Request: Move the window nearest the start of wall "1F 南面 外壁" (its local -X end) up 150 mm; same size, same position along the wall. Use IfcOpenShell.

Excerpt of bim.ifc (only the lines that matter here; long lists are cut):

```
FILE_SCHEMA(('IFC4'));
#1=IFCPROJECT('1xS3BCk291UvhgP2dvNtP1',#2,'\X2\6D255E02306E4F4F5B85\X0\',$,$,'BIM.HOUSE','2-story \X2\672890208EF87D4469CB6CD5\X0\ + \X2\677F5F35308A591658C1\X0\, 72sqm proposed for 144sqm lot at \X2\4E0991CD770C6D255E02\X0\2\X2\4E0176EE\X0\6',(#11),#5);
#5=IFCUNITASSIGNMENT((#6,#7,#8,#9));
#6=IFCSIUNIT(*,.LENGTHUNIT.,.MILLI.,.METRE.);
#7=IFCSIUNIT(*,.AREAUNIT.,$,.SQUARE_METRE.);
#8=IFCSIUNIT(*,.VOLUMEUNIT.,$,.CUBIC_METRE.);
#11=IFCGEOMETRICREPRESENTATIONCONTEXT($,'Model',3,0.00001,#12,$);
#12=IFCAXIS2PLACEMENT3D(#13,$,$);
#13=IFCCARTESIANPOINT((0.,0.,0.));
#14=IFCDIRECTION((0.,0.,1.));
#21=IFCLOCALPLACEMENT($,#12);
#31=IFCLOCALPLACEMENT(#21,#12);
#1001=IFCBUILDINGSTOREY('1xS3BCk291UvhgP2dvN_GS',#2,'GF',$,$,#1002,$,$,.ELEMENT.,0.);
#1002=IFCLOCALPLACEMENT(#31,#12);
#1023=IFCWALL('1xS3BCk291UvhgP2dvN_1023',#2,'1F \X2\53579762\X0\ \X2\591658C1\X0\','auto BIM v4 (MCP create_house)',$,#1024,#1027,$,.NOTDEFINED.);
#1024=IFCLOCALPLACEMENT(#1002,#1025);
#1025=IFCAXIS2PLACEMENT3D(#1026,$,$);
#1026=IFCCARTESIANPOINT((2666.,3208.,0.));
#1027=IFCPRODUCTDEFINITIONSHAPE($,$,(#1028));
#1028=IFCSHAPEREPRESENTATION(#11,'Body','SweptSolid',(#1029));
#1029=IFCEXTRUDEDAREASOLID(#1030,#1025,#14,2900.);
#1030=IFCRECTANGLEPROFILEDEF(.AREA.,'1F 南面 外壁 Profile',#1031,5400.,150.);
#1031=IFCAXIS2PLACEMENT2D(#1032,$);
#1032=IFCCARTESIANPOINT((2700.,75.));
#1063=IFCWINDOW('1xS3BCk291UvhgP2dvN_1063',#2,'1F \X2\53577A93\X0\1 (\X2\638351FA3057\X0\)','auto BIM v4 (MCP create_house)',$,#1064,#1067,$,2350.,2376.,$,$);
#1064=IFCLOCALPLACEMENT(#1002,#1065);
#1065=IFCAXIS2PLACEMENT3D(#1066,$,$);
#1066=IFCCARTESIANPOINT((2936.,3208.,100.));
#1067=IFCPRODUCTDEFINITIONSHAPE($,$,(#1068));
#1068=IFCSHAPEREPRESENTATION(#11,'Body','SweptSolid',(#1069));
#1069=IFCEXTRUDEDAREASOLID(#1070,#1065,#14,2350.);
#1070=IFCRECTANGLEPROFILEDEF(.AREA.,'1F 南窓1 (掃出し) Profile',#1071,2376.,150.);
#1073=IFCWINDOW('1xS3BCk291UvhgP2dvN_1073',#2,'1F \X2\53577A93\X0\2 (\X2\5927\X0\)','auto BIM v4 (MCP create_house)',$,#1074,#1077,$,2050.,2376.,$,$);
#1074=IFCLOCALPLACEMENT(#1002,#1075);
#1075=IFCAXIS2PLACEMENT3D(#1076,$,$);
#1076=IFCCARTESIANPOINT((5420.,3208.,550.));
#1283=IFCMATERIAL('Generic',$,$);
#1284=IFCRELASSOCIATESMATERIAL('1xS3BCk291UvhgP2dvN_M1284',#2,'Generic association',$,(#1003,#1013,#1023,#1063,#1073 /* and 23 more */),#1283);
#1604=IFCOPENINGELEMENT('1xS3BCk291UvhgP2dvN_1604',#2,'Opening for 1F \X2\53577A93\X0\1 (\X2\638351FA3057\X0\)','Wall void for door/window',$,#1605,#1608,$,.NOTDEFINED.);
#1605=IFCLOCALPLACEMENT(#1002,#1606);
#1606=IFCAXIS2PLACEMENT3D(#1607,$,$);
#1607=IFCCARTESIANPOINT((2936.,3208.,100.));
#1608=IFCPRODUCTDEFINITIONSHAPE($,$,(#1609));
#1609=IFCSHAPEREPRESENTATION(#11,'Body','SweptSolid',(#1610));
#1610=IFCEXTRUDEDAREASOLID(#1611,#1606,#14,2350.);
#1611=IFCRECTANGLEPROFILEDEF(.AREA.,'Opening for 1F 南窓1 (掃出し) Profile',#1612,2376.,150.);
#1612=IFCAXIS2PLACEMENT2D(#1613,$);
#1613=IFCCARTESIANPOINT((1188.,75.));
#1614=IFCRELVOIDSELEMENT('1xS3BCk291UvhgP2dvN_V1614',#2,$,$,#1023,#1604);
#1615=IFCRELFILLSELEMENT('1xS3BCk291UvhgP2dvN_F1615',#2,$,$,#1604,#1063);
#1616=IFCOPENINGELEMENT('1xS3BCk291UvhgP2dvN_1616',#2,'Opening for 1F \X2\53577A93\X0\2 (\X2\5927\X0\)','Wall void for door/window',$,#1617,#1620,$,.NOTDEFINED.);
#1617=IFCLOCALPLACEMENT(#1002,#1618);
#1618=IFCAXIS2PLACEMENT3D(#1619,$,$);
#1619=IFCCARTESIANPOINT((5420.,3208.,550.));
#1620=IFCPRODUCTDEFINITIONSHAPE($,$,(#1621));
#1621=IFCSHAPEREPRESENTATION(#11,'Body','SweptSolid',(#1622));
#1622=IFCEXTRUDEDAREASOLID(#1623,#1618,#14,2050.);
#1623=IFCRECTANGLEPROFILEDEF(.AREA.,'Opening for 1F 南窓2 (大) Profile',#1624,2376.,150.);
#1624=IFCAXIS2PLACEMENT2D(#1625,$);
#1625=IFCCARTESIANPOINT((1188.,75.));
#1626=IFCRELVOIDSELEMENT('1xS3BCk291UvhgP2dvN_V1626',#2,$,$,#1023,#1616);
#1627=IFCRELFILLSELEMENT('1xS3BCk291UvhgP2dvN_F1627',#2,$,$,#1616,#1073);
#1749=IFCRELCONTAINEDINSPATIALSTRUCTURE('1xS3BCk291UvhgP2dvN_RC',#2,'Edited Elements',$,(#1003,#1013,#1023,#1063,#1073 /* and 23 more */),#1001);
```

```python
import numpy as np
import ifcopenshell
import ifcopenshell.api.geometry
import ifcopenshell.util.placement
import ifcopenshell.util.unit

model = ifcopenshell.open("bim.ifc")
unit_scale = ifcopenshell.util.unit.calculate_unit_scale(model)

window = model.by_id(1063)
opening = window.FillsVoids[0].RelatingOpeningElement
dz = 150.0

shift = np.array([0.0, 0.0, dz])
# The window is not placed relative to its opening, so move both.
for product in (opening, window):
    matrix = ifcopenshell.util.placement.get_local_placement(product.ObjectPlacement)
    matrix[:3, 3] += shift
    ifcopenshell.api.geometry.edit_object_placement(model, product=product, matrix=matrix, is_si=False)

print(f"moved by {dz * unit_scale:+.3f} m")

model.write("bim_edited.ifc")
```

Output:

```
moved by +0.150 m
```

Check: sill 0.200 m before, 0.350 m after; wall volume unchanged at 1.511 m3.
